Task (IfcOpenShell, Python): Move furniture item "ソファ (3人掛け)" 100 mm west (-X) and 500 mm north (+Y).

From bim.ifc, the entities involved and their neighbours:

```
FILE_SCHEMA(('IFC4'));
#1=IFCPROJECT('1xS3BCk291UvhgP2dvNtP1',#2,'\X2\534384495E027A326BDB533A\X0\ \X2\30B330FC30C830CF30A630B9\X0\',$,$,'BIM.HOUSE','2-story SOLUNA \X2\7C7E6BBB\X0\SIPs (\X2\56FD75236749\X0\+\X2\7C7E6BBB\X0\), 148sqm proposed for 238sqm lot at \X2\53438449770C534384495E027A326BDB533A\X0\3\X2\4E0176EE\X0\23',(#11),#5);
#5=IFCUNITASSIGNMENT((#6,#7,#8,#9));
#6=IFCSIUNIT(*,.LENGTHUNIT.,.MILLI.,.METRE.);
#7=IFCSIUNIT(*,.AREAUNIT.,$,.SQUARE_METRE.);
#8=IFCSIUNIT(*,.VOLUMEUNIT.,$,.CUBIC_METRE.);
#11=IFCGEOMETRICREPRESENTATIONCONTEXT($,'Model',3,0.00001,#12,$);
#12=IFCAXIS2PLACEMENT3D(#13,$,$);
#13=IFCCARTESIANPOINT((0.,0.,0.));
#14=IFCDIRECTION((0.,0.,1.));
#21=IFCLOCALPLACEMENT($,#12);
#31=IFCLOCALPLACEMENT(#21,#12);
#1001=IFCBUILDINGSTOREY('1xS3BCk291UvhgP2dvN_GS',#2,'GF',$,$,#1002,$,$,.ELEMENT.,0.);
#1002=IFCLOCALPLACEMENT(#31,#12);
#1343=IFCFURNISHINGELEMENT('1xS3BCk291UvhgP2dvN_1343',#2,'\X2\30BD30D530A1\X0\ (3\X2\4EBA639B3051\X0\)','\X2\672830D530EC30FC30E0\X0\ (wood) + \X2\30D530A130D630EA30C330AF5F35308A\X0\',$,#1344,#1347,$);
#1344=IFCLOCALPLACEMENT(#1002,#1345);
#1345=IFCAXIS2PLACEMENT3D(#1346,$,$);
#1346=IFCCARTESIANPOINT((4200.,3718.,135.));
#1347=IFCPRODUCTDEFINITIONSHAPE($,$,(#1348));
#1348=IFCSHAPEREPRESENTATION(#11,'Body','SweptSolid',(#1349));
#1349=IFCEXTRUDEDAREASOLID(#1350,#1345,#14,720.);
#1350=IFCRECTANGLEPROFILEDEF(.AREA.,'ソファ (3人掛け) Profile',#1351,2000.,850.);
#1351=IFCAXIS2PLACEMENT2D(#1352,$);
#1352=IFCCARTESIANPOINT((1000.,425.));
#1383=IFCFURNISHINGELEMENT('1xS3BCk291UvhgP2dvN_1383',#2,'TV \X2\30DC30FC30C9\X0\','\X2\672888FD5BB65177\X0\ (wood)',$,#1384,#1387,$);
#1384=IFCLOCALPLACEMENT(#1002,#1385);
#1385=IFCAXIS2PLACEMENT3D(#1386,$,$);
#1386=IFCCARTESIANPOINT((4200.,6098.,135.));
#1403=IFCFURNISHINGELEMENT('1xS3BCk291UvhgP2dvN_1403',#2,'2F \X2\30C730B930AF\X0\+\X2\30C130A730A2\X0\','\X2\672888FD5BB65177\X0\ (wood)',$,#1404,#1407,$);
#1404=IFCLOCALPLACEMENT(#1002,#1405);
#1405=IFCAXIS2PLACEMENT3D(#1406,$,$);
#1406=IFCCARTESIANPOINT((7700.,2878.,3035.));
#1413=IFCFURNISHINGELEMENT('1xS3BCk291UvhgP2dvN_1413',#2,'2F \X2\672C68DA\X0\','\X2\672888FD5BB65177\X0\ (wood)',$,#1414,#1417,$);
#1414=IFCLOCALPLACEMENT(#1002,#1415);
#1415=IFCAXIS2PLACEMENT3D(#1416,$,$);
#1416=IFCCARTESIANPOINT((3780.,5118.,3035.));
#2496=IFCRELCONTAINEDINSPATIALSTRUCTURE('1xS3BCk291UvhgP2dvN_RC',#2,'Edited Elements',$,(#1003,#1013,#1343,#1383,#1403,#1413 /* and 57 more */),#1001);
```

```python
import ifcopenshell
import ifcopenshell.api.geometry
import ifcopenshell.util.placement
import ifcopenshell.util.unit

model = ifcopenshell.open("bim.ifc")
unit_scale = ifcopenshell.util.unit.calculate_unit_scale(model)

item = model.by_id(1343)
matrix = ifcopenshell.util.placement.get_local_placement(item.ObjectPlacement)
matrix[0, 3] -= 0.1 / unit_scale
matrix[1, 3] += 0.5 / unit_scale
ifcopenshell.api.geometry.edit_object_placement(model, product=item, matrix=matrix, is_si=False)

print(ifcopenshell.util.placement.get_local_placement(item.ObjectPlacement).round(3) + 0.0)

model.write("bim_rev.ifc")
```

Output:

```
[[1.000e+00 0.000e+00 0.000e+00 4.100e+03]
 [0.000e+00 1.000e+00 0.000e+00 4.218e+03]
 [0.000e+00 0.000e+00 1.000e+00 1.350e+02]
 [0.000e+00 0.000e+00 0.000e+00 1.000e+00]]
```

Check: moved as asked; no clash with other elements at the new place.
